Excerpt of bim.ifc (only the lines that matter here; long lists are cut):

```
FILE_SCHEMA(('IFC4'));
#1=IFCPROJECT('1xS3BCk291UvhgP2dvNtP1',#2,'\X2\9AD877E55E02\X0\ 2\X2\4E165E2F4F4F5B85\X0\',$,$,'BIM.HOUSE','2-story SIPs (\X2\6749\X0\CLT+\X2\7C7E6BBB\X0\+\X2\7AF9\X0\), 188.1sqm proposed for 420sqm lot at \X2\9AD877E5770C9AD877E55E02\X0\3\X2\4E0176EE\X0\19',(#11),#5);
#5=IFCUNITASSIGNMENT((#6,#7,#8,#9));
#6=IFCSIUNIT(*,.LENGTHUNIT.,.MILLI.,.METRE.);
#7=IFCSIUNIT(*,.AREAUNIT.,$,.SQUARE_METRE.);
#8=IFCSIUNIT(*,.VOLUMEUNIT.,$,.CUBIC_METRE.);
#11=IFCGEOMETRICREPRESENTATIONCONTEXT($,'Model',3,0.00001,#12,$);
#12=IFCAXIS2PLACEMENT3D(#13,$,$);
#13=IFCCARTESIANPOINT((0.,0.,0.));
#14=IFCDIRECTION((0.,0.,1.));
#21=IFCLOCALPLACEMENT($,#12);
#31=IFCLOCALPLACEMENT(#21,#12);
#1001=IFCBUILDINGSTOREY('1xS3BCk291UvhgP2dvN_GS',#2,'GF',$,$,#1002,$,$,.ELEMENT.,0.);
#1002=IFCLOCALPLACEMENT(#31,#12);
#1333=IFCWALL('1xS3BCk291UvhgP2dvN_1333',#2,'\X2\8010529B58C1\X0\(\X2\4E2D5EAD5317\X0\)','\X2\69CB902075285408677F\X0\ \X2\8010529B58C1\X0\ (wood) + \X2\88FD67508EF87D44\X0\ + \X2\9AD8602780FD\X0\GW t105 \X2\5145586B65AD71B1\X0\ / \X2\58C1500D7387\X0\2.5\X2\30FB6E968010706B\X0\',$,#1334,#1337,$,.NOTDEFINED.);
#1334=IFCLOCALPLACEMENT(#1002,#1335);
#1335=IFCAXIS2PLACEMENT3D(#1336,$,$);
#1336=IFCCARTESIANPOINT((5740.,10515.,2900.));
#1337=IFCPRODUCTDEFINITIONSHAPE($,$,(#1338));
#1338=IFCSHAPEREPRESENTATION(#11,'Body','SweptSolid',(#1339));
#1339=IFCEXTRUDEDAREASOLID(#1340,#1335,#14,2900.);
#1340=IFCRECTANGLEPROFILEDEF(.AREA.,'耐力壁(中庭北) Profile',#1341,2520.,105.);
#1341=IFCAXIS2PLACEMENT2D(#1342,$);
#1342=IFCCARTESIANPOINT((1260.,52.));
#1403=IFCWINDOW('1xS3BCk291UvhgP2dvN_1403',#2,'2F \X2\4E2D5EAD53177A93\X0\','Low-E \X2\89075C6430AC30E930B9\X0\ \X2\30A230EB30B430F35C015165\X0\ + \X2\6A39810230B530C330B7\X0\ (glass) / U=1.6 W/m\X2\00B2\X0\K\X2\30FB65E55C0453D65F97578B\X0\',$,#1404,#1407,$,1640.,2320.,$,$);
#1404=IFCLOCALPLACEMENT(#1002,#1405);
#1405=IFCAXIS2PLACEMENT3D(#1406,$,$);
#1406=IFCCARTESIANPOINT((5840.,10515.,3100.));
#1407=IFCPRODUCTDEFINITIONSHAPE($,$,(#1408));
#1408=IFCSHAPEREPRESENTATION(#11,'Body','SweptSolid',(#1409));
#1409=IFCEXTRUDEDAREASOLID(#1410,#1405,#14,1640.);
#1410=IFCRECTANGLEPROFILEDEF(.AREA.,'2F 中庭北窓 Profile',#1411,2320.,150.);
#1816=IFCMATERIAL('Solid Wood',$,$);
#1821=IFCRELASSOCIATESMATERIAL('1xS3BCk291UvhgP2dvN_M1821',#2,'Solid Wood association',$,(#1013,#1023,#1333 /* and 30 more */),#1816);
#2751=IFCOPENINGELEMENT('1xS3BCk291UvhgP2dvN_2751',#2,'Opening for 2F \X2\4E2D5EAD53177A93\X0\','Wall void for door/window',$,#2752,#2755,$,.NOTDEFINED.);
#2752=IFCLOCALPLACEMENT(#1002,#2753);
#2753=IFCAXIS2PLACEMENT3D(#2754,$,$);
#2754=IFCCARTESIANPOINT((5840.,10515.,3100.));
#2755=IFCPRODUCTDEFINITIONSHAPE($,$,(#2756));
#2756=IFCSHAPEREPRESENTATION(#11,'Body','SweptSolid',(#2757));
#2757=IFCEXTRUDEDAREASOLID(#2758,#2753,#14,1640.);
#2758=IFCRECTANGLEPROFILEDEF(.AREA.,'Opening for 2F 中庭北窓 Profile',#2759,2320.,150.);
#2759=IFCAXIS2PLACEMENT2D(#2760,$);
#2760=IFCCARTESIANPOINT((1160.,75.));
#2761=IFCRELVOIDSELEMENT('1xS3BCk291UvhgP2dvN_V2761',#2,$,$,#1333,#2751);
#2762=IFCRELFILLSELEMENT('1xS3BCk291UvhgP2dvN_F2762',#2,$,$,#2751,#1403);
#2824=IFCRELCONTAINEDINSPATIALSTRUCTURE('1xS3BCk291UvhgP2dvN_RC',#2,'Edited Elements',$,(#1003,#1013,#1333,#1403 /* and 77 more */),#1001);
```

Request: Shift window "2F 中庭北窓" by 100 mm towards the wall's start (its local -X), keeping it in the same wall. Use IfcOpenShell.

```python
import ifcopenshell
import ifcopenshell.api.geometry
import ifcopenshell.util.placement
import ifcopenshell.util.unit

model = ifcopenshell.open("bim.ifc")
unit_scale = ifcopenshell.util.unit.calculate_unit_scale(model)

window = model.by_guid("1xS3BCk291UvhgP2dvN_1403")
opening = window.FillsVoids[0].RelatingOpeningElement
wall = opening.VoidsElements[0].RelatingBuildingElement

wall_matrix = ifcopenshell.util.placement.get_local_placement(wall.ObjectPlacement)
shift = wall_matrix[:3, 0] * -0.1 / unit_scale
before = ifcopenshell.util.placement.get_local_placement(window.ObjectPlacement)[:3, 3].copy()

# The window is not placed relative to its opening, so move both.
for product in (opening, window):
    matrix = ifcopenshell.util.placement.get_local_placement(product.ObjectPlacement)
    matrix[:3, 3] += shift
    ifcopenshell.api.geometry.edit_object_placement(model, product=product, matrix=matrix, is_si=False)

after = ifcopenshell.util.placement.get_local_placement(window.ObjectPlacement)[:3, 3]
print("window moved by", (after - before).round(3) + 0.0)

model.write("bim_rev.ifc")
```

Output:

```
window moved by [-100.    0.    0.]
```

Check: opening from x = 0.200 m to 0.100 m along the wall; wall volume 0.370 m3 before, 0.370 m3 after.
